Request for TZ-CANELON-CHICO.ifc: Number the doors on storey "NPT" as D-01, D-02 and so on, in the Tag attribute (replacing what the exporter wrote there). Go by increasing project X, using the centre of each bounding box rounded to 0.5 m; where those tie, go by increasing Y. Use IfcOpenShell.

First a look at what the model holds.

```python
import ifcopenshell
import ifcopenshell.util.element
import ifcopenshell.util.placement

model = ifcopenshell.open("TZ-CANELON-CHICO.ifc")
print(model.schema)
storey = next(s for s in model.by_type("IfcBuildingStorey") if s.Name == "NPT")
doors = [e for e in ifcopenshell.util.element.get_decomposition(storey) if e.is_a("IfcDoor")]
for e in sorted(doors, key=lambda e: e.id()):
    origin = ifcopenshell.util.placement.get_local_placement(e.ObjectPlacement)[:3, 3]
    print(e.id(), e.Tag, e.Name, origin.round(2) + 0.0, sep=" | ")
```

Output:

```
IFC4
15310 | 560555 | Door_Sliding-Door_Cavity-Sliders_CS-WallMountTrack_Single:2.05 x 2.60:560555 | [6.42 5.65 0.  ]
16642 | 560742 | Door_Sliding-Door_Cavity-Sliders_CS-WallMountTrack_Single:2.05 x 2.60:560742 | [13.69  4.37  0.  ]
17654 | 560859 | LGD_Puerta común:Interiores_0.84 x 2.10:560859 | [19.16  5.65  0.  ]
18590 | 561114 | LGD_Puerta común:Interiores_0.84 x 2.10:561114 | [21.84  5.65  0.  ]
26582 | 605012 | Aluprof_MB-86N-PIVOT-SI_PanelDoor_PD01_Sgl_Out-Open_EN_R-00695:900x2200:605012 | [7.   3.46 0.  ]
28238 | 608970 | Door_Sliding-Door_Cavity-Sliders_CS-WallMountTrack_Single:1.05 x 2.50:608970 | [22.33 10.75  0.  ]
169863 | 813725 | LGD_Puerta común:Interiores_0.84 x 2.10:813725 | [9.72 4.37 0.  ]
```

```python
import ifcopenshell
import ifcopenshell.geom
import ifcopenshell.util.element
import ifcopenshell.util.shape

model = ifcopenshell.open("TZ-CANELON-CHICO.ifc")
settings = ifcopenshell.geom.settings()
settings.set("use-world-coords", True)


def centre(element):
    shape = ifcopenshell.geom.create_shape(settings, element)
    return ifcopenshell.util.shape.get_bbox_centroid(shape.geometry)


storey = next(s for s in model.by_type("IfcBuildingStorey") if s.Name == "NPT")
doors = [e for e in ifcopenshell.util.element.get_decomposition(storey) if e.is_a("IfcDoor")]

# Insertion points can sit at a corner or the storey origin, so sort by the geometry (in metres).
centres = {e: centre(e) for e in doors}
doors.sort(key=lambda e: (round(centres[e][0] / 0.5), centres[e][1]))

for i, e in enumerate(doors, start=1):
    number = f"D-{i:02d}"
    e.Tag = number
    print(e.id(), number)

model.write("TZ-CANELON-CHICO-out.ifc")
```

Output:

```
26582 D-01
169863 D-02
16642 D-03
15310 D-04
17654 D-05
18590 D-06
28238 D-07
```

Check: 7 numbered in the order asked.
